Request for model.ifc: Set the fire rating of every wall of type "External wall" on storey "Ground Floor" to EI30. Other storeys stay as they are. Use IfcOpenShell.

First a look at what the model holds.

```python
import ifcopenshell
import ifcopenshell.util.element

model = ifcopenshell.open("model.ifc")
print(model.schema)
storey = next(s for s in model.by_type("IfcBuildingStorey") if s.Name == "Ground Floor")
walls = [e for e in ifcopenshell.util.element.get_decomposition(storey) if e.is_a("IfcWall")]
seen = {}
for e in walls:
    element_type = ifcopenshell.util.element.get_type(e)
    key = (element_type.Name if element_type != e and element_type else None, ifcopenshell.util.element.get_pset(e, "Pset_WallCommon", "FireRating"))
    seen[key] = seen.get(key, 0) + 1
for (name, value), count in sorted(seen.items(), key=str):
    print(count, "x", name, "|", value)
```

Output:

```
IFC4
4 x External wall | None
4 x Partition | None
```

```python
import ifcopenshell
import ifcopenshell.api.pset
import ifcopenshell.util.element

model = ifcopenshell.open("model.ifc")

storey = next(s for s in model.by_type("IfcBuildingStorey") if s.Name == "Ground Floor")
walls = [e for e in ifcopenshell.util.element.get_decomposition(storey) if e.is_a("IfcWall")]

count = 0
for e in walls:
    element_type = ifcopenshell.util.element.get_type(e)
    if element_type in (None, e) or element_type.Name != "External wall":
        continue
    # add_pset returns the element's existing set when there is one.
    pset = ifcopenshell.api.pset.add_pset(model, product=e, name="Pset_WallCommon")
    ifcopenshell.api.pset.edit_pset(model, pset=pset, properties={"FireRating": "EI30"})
    count += 1

print(count, "walls updated")

model.write("model_edited.ifc")
```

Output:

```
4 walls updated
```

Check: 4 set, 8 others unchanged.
